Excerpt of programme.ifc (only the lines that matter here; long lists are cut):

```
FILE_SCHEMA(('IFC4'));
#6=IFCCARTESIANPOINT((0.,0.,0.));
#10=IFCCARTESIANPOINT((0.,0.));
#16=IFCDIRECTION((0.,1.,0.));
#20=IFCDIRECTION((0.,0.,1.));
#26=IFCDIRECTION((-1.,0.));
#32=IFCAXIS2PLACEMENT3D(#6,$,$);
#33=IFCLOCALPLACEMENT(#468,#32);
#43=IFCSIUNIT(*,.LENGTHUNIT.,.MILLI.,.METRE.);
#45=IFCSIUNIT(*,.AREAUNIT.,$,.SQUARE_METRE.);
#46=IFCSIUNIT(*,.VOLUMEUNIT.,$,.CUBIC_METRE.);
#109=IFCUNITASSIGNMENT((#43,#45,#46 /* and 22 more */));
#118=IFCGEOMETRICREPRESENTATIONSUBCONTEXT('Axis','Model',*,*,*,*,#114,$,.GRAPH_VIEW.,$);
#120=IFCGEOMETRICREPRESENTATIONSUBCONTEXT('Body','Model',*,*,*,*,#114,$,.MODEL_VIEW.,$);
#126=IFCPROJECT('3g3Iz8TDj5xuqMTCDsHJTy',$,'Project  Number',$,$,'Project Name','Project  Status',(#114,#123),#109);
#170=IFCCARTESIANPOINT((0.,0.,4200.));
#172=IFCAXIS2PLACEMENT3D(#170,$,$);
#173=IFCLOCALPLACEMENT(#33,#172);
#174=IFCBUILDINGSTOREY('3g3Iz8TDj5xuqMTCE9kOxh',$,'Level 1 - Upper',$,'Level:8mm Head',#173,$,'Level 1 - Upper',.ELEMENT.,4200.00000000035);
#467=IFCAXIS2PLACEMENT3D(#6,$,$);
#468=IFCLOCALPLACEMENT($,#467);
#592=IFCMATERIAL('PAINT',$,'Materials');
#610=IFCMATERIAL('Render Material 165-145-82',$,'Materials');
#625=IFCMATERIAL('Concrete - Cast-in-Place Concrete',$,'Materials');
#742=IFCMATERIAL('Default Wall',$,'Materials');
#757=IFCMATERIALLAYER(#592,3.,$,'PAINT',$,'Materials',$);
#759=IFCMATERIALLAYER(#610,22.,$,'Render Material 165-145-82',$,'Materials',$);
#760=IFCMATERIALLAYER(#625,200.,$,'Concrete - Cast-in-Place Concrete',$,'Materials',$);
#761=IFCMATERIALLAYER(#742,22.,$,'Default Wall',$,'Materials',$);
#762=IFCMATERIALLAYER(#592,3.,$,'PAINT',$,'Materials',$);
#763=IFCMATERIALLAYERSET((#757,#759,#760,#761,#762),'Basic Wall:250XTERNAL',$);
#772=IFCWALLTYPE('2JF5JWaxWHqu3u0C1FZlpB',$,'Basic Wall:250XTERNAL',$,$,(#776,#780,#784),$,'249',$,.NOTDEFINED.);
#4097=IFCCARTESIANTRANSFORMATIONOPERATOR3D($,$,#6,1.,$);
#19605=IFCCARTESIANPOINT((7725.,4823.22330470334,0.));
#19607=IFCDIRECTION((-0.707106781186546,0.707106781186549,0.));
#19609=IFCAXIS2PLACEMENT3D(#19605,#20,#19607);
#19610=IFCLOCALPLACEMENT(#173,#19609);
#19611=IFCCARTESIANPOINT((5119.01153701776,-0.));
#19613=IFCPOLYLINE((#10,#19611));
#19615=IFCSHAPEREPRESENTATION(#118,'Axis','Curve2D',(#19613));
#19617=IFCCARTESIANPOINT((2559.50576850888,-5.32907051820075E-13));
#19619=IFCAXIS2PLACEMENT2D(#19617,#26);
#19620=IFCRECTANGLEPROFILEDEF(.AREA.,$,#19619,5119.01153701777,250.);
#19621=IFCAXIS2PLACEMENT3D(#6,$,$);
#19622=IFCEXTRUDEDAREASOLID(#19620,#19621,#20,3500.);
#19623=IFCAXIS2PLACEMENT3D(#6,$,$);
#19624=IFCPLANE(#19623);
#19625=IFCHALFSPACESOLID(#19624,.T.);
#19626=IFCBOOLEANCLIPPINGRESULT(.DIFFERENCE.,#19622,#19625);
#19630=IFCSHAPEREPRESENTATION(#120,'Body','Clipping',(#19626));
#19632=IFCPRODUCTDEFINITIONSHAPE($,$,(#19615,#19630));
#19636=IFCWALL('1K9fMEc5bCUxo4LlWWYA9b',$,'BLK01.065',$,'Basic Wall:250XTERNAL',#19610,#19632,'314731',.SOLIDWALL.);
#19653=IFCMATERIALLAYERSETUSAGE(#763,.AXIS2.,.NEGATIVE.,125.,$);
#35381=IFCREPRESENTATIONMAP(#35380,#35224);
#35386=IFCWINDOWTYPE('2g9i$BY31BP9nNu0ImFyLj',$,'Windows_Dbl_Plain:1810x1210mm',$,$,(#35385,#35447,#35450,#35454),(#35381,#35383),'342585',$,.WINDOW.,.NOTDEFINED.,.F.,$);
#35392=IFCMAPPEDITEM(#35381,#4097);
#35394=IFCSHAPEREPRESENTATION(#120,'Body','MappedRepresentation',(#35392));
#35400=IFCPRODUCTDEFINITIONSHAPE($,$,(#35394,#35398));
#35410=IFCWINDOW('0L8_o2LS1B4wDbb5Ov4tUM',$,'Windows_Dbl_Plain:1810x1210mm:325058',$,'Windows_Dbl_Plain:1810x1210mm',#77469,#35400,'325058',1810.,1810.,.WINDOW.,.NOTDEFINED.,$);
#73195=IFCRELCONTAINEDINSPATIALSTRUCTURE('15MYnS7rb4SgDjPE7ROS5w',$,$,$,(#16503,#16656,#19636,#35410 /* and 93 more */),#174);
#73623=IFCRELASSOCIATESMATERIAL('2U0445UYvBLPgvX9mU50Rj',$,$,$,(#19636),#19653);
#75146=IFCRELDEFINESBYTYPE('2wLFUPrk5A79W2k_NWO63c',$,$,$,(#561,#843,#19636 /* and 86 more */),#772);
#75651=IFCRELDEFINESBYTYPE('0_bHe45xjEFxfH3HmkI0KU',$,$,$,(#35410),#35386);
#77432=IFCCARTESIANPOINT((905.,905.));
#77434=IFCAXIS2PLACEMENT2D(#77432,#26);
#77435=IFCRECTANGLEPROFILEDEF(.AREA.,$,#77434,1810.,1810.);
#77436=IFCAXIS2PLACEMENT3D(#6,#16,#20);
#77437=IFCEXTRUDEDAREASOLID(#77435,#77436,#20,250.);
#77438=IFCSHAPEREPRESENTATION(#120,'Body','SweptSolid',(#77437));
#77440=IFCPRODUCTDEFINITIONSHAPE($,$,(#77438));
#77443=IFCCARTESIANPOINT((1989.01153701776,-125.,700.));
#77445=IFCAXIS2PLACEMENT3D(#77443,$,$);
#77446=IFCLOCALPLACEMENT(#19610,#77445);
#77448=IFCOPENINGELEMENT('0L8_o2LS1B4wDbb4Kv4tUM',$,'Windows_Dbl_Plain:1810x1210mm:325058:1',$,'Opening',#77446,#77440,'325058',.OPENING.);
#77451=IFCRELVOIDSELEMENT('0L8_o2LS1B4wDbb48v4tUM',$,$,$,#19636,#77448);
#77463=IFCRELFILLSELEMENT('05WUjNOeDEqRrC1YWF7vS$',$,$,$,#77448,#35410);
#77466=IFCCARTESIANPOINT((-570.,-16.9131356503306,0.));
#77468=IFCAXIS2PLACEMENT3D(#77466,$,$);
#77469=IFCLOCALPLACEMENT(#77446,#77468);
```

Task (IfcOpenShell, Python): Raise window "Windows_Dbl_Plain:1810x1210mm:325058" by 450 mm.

```python
import numpy as np
import ifcopenshell
import ifcopenshell.api.geometry
import ifcopenshell.util.placement
import ifcopenshell.util.unit

model = ifcopenshell.open("programme.ifc")
unit_scale = ifcopenshell.util.unit.calculate_unit_scale(model)

window = model.by_guid("0L8_o2LS1B4wDbb5Ov4tUM")
opening = window.FillsVoids[0].RelatingOpeningElement
dz = 450.0

shift = np.array([0.0, 0.0, dz])
# The window is placed relative to its opening, so it follows when the opening moves.
matrix = ifcopenshell.util.placement.get_local_placement(opening.ObjectPlacement)
matrix[:3, 3] += shift
ifcopenshell.api.geometry.edit_object_placement(
    model, product=opening, matrix=matrix, is_si=False, should_transform_children=True
)

print(f"moved by {dz * unit_scale:+.3f} m")

model.write("programme_v2.ifc")
```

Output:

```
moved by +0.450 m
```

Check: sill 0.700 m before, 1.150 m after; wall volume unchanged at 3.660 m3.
